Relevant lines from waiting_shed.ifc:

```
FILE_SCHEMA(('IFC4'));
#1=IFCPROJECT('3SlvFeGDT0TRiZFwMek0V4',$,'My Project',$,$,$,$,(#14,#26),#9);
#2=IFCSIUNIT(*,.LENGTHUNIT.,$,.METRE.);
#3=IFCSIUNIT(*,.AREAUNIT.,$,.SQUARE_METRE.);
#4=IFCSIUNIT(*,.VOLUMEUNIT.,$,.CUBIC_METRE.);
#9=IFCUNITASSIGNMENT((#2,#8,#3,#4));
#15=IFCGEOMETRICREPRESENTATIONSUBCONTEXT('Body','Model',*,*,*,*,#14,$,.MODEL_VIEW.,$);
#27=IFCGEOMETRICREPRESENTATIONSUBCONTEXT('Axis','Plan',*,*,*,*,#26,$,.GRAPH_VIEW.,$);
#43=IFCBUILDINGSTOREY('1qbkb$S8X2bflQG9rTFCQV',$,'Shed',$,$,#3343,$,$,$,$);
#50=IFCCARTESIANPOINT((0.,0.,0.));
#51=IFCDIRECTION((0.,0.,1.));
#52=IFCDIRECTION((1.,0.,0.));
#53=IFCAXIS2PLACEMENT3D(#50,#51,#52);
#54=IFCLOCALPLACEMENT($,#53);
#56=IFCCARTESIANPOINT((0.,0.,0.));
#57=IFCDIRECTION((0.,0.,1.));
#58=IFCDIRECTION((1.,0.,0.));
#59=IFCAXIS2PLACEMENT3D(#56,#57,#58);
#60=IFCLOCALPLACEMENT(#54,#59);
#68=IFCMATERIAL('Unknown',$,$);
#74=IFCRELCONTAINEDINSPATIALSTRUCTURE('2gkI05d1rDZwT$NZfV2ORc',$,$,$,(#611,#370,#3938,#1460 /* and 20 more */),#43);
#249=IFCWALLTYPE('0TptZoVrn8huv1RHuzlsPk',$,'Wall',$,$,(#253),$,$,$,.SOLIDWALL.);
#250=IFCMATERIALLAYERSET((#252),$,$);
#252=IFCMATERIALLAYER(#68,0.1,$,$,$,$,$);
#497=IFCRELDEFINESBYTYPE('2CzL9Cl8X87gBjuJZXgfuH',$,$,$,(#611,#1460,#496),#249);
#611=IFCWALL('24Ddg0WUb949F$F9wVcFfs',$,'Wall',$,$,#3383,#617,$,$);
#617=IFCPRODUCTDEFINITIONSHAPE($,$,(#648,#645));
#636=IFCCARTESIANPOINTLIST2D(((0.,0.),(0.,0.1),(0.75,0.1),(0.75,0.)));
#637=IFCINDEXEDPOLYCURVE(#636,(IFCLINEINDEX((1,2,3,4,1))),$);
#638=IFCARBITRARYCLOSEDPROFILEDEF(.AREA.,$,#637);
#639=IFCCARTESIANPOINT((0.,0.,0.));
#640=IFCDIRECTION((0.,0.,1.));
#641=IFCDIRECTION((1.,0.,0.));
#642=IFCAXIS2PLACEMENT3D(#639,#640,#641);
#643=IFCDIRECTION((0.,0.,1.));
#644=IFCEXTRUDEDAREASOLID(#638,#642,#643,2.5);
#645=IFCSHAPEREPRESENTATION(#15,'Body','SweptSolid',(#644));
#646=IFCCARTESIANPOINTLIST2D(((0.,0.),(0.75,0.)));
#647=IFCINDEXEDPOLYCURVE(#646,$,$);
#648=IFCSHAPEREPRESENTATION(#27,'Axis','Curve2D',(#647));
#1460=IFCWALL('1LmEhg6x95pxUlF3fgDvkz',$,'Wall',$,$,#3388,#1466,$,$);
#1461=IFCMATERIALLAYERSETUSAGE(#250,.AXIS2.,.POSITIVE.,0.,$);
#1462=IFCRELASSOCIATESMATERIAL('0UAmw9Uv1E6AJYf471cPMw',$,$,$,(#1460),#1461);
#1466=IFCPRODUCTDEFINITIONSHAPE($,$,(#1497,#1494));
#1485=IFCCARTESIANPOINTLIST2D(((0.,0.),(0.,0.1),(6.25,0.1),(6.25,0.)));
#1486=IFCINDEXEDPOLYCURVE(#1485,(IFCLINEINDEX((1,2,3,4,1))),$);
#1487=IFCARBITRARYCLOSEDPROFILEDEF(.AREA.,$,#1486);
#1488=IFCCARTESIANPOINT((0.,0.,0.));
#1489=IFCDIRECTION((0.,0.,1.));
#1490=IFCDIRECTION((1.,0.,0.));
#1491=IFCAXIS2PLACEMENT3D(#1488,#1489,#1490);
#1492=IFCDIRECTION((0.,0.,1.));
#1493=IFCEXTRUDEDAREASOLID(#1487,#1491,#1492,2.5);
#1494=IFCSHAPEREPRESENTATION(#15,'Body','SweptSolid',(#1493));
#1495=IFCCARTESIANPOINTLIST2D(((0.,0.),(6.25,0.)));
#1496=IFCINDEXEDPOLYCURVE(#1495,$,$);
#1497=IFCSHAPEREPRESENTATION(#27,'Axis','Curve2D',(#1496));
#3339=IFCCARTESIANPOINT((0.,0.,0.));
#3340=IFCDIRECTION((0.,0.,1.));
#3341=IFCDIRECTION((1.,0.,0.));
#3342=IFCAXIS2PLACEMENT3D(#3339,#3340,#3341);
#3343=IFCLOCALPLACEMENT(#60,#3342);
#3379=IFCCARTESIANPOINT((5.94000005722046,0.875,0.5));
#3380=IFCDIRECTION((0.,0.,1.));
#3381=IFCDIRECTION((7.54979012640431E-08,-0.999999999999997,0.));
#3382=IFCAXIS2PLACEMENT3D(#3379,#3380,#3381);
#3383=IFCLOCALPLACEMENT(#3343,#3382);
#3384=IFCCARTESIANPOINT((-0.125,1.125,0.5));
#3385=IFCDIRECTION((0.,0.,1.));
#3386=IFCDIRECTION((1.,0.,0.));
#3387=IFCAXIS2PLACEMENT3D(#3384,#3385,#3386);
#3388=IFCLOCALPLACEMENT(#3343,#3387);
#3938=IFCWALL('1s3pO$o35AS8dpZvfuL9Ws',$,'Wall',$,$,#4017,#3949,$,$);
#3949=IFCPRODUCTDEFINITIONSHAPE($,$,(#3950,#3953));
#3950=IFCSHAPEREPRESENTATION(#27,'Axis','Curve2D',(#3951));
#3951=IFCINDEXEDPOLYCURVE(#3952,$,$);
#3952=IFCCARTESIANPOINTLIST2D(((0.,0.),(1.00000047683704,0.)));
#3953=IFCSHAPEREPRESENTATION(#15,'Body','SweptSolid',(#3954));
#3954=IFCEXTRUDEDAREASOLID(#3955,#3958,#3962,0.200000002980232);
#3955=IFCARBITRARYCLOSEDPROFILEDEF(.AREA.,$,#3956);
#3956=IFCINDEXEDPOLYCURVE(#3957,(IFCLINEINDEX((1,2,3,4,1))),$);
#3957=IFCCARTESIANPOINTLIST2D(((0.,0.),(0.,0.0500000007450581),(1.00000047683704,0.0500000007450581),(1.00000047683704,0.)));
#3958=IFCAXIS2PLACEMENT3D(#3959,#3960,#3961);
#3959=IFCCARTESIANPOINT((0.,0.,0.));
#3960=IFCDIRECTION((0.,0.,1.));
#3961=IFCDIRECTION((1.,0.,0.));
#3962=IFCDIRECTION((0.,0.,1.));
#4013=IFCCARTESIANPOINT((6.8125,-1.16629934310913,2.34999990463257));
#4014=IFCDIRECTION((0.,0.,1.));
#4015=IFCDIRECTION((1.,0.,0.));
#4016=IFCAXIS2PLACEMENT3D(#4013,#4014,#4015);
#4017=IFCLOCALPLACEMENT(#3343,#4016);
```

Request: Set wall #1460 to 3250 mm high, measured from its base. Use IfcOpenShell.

```python
import ifcopenshell
import ifcopenshell.geom
import ifcopenshell.util.representation
import ifcopenshell.util.shape
import ifcopenshell.util.unit

model = ifcopenshell.open("waiting_shed.ifc")
unit_scale = ifcopenshell.util.unit.calculate_unit_scale(model)
settings = ifcopenshell.geom.settings()


def volume(element):
    """Net volume in cubic metres, openings subtracted."""
    shape = ifcopenshell.geom.create_shape(settings, element)
    return ifcopenshell.util.shape.get_volume(shape.geometry)


wall = model.by_id(1460)
before = volume(wall)

body = ifcopenshell.util.representation.get_representation(wall, "Model", "Body")
solid = body.Items[0]
old_height = solid.Depth
solid.Depth = 3.25 / unit_scale
after = volume(wall)

print(f"height {old_height:g} -> {solid.Depth:g}, volume {before:.3f} -> {after:.3f} m3")

model.write("waiting_shed_updated.ifc")
```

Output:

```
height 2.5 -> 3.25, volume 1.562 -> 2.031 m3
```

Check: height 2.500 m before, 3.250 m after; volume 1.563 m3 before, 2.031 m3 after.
